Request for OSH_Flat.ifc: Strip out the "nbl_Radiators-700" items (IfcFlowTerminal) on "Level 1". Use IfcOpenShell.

First a look at what the model holds.

```python
import ifcopenshell
import ifcopenshell.util.element

model = ifcopenshell.open("OSH_Flat.ifc")
print(model.schema)
storey = next(s for s in model.by_type("IfcBuildingStorey") if s.Name == "Level 1")
terminals = [e for e in ifcopenshell.util.element.get_decomposition(storey) if e.is_a("IfcFlowTerminal")]
seen = {}
for e in terminals:
    element_type = ifcopenshell.util.element.get_type(e)
    name = element_type.Name if element_type not in (None, e) else None
    seen[name] = seen.get(name, 0) + 1
for name, count in sorted(seen.items(), key=str):
    print(count, "x", name)
```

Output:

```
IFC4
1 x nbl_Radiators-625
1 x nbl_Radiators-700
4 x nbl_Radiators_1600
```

```python
import ifcopenshell
import ifcopenshell.api.root
import ifcopenshell.util.element

model = ifcopenshell.open("OSH_Flat.ifc")

storey = next(s for s in model.by_type("IfcBuildingStorey") if s.Name == "Level 1")
terminals = [e for e in ifcopenshell.util.element.get_decomposition(storey) if e.is_a("IfcFlowTerminal")]
targets = [e for e in terminals if (t := ifcopenshell.util.element.get_type(e)) not in (None, e) and t.Name == "nbl_Radiators-700"]

for e in targets:
    ifcopenshell.api.root.remove_product(model, product=e)
print(len(targets), "removed")

model.write("OSH_Flat_edited.ifc")
```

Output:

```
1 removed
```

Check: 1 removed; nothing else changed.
